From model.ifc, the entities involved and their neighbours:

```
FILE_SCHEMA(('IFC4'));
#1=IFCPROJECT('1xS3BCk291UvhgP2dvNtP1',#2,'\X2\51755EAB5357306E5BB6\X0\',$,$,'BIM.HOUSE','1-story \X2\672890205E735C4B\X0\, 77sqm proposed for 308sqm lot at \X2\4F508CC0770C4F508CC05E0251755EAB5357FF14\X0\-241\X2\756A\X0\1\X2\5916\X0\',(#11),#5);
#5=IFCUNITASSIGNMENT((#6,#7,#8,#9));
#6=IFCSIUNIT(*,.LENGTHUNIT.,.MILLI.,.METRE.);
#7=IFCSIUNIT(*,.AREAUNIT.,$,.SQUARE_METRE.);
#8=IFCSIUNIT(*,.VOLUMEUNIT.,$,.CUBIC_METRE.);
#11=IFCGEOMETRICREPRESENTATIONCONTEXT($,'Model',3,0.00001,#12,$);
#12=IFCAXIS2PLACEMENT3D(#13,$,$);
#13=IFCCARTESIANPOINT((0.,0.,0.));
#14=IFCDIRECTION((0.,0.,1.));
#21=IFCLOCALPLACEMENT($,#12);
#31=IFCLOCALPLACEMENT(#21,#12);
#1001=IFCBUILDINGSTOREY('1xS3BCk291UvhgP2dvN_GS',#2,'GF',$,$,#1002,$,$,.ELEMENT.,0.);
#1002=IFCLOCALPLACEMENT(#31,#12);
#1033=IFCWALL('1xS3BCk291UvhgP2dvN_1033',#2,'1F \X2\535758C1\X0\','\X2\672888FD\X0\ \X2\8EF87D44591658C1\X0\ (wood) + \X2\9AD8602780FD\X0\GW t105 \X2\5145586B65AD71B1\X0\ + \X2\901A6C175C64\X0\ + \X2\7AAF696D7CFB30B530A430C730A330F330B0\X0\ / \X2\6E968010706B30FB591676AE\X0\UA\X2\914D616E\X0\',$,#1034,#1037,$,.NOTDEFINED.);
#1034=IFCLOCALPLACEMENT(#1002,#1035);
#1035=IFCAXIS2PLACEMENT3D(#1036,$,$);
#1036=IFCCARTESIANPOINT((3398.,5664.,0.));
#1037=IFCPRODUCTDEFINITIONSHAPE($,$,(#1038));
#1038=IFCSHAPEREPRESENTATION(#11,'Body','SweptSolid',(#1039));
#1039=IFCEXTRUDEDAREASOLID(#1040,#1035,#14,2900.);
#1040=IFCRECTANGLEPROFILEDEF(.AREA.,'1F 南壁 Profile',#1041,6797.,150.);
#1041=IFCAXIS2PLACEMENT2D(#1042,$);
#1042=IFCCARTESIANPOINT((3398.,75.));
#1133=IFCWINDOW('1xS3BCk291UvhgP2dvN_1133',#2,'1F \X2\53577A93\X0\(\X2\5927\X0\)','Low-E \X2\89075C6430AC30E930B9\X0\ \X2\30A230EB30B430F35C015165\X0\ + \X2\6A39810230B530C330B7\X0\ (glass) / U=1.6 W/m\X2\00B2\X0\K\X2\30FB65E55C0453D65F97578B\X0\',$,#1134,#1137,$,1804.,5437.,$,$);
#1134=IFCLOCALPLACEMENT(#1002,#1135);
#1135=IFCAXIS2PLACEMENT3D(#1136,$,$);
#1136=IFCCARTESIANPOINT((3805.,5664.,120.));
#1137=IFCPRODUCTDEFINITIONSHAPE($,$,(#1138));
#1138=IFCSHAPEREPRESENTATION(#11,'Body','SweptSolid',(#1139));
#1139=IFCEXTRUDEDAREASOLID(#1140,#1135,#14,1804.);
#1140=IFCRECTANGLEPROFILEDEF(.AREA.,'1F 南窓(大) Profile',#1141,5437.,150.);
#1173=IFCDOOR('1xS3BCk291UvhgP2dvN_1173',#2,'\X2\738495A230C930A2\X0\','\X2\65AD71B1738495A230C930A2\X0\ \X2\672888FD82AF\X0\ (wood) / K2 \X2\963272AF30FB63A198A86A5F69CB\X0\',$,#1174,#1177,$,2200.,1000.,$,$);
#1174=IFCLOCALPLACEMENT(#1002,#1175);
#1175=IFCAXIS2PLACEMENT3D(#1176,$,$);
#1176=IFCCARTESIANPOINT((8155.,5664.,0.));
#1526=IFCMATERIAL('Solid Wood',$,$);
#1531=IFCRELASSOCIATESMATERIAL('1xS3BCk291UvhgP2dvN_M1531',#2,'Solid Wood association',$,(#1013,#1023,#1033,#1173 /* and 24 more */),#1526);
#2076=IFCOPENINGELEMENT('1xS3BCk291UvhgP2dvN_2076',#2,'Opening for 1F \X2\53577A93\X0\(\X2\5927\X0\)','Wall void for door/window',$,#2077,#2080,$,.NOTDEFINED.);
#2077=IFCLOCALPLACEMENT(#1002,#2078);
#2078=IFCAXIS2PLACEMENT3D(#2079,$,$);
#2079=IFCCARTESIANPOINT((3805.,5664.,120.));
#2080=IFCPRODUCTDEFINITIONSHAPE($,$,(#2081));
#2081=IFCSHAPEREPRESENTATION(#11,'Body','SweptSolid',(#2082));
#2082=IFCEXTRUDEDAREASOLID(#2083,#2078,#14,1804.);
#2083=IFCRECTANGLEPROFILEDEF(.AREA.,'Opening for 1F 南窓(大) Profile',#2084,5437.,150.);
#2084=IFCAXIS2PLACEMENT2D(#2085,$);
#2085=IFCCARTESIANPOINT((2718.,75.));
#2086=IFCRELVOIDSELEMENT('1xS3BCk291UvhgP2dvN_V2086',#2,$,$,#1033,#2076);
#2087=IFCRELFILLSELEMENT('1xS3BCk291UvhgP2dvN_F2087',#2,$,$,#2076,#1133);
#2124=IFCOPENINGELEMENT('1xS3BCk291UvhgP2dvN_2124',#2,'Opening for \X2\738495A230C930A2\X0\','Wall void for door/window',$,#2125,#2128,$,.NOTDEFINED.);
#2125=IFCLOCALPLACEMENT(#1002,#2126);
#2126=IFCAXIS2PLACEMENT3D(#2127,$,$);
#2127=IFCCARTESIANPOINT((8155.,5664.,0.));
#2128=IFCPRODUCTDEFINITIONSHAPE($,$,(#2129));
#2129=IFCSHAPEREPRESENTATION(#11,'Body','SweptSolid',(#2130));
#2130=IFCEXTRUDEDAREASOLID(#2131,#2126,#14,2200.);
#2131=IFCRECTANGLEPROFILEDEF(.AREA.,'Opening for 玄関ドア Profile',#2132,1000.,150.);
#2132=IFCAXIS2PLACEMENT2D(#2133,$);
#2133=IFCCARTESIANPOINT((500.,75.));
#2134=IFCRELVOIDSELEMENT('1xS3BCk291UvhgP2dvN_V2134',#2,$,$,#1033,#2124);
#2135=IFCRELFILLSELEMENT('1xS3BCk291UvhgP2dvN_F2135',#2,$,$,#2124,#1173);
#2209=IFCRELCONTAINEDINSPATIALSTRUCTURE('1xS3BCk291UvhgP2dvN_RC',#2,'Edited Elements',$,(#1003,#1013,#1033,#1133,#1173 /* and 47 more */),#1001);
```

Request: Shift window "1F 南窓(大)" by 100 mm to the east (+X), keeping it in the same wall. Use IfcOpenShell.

```python
import ifcopenshell
import ifcopenshell.api.geometry
import ifcopenshell.util.placement
import ifcopenshell.util.unit

model = ifcopenshell.open("model.ifc")
unit_scale = ifcopenshell.util.unit.calculate_unit_scale(model)

window = model.by_guid("1xS3BCk291UvhgP2dvN_1133")
opening = window.FillsVoids[0].RelatingOpeningElement
wall = opening.VoidsElements[0].RelatingBuildingElement

wall_matrix = ifcopenshell.util.placement.get_local_placement(wall.ObjectPlacement)
shift = wall_matrix[:3, 0] * 0.1 / unit_scale
before = ifcopenshell.util.placement.get_local_placement(window.ObjectPlacement)[:3, 3].copy()

# The window is not placed relative to its opening, so move both.
for product in (opening, window):
    matrix = ifcopenshell.util.placement.get_local_placement(product.ObjectPlacement)
    matrix[:3, 3] += shift
    ifcopenshell.api.geometry.edit_object_placement(model, product=product, matrix=matrix, is_si=False)

after = ifcopenshell.util.placement.get_local_placement(window.ObjectPlacement)[:3, 3]
print("window moved by", (after - before).round(3) + 0.0)

model.write("model_v2.ifc")
```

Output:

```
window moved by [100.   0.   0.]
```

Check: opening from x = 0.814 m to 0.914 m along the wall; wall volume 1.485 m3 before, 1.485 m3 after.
